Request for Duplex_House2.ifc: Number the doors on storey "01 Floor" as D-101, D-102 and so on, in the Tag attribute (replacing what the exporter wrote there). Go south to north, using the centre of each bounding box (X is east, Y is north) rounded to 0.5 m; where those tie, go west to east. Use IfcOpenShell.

First a look at what the model holds.

```python
import ifcopenshell
import ifcopenshell.util.element
import ifcopenshell.util.placement

model = ifcopenshell.open("Duplex_House2.ifc")
print(model.schema)
storey = next(s for s in model.by_type("IfcBuildingStorey") if s.Name == "01 Floor")
doors = [e for e in ifcopenshell.util.element.get_decomposition(storey) if e.is_a("IfcDoor")]
for e in sorted(doors, key=lambda e: e.id()):
    origin = ifcopenshell.util.placement.get_local_placement(e.ObjectPlacement)[:3, 3]
    print(e.id(), e.Tag, e.Name, origin.round(2) + 0.0, sep=" | ")
```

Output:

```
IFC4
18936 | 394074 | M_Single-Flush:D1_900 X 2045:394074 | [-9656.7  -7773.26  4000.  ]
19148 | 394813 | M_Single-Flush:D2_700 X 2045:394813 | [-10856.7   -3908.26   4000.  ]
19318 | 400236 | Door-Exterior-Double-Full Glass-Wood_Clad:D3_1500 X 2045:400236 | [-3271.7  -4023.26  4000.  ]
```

```python
import ifcopenshell
import ifcopenshell.geom
import ifcopenshell.util.element
import ifcopenshell.util.shape

model = ifcopenshell.open("Duplex_House2.ifc")
settings = ifcopenshell.geom.settings()
settings.set("use-world-coords", True)


def centre(element):
    shape = ifcopenshell.geom.create_shape(settings, element)
    return ifcopenshell.util.shape.get_bbox_centroid(shape.geometry)


storey = next(s for s in model.by_type("IfcBuildingStorey") if s.Name == "01 Floor")
doors = [e for e in ifcopenshell.util.element.get_decomposition(storey) if e.is_a("IfcDoor")]

# Insertion points can sit at a corner or the storey origin, so sort by the geometry (in metres).
centres = {e: centre(e) for e in doors}
doors.sort(key=lambda e: (round(centres[e][1] / 0.5), centres[e][0]))

for i, e in enumerate(doors, start=1):
    number = f"D-1{i:02d}"
    e.Tag = number
    print(e.id(), number)

model.write("Duplex_House2-out.ifc")
```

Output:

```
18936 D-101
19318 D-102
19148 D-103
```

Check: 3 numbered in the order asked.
